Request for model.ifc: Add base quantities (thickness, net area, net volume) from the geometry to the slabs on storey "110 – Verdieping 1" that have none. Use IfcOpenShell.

First a look at what the model holds.

```python
import ifcopenshell
import ifcopenshell.util.element
import ifcopenshell.util.unit

model = ifcopenshell.open("model.ifc")
print(model.schema)
for unit_type in ("LENGTHUNIT", "AREAUNIT", "VOLUMEUNIT"):
    print(unit_type, ifcopenshell.util.unit.calculate_unit_scale(model, unit_type))
storey = next(s for s in model.by_type("IfcBuildingStorey") if s.Name == "110 – Verdieping 1")
slabs = [e for e in ifcopenshell.util.element.get_decomposition(storey) if e.is_a("IfcSlab")]
for e in sorted(slabs, key=lambda e: e.id()):
    print(e.id(), e.is_a(), e.Name, list(ifcopenshell.util.element.get_psets(e, qtos_only=True)), sep=" | ")
```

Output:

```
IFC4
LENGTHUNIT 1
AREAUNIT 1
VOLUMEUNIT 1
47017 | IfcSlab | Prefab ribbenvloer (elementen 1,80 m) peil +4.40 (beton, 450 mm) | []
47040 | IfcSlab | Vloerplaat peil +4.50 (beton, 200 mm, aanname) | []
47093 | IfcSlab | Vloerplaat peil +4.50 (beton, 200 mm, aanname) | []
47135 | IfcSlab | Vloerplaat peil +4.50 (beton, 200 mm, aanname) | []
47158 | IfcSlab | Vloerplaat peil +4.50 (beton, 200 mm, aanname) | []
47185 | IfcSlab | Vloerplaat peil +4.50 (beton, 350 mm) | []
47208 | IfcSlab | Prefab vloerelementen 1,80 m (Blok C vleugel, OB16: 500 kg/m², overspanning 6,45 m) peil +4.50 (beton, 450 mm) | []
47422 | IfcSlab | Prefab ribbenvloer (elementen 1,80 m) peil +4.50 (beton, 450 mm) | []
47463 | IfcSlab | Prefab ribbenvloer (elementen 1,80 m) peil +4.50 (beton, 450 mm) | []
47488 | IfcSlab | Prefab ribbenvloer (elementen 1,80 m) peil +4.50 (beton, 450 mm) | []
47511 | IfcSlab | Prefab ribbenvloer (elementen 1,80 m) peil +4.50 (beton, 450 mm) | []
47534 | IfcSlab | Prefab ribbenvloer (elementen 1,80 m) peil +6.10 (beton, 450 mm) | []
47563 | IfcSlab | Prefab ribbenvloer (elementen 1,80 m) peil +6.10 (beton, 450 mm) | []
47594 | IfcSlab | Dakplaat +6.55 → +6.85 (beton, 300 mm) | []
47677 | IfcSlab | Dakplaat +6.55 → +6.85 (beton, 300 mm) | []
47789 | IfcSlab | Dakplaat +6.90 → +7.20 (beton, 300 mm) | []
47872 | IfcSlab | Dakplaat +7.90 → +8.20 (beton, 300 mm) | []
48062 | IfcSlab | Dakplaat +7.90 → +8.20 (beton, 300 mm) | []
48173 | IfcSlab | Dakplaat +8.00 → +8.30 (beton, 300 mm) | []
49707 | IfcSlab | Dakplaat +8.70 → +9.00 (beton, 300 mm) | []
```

```python
import ifcopenshell
import ifcopenshell.api.pset
import ifcopenshell.geom
import ifcopenshell.util.element
import ifcopenshell.util.shape
import ifcopenshell.util.unit

model = ifcopenshell.open("model.ifc")
unit_scale = ifcopenshell.util.unit.calculate_unit_scale(model)
area_scale = ifcopenshell.util.unit.calculate_unit_scale(model, "AREAUNIT")
volume_scale = ifcopenshell.util.unit.calculate_unit_scale(model, "VOLUMEUNIT")
settings = ifcopenshell.geom.settings()

storey = next(s for s in model.by_type("IfcBuildingStorey") if s.Name == "110 – Verdieping 1")
slabs = [e for e in ifcopenshell.util.element.get_decomposition(storey) if e.is_a("IfcSlab")]

for e in sorted(slabs, key=lambda e: e.id()):
    if ifcopenshell.util.element.get_psets(e, qtos_only=True, should_inherit=False):
        continue
    # Geometry comes back in metres, in the element's own axes.
    shape = ifcopenshell.geom.create_shape(settings, e)
    values = {
        "Width": ifcopenshell.util.shape.get_z(shape.geometry) / unit_scale,
        "NetArea": ifcopenshell.util.shape.get_footprint_area(shape.geometry) / area_scale,
        "NetVolume": ifcopenshell.util.shape.get_volume(shape.geometry) / volume_scale,
    }
    qto = ifcopenshell.api.pset.add_qto(model, product=e, name="Qto_SlabBaseQuantities")
    ifcopenshell.api.pset.edit_qto(model, qto=qto, properties=values)
    print(e.id(), {k: round(v, 3) for k, v in values.items()})

model.write("model_updated.ifc")
```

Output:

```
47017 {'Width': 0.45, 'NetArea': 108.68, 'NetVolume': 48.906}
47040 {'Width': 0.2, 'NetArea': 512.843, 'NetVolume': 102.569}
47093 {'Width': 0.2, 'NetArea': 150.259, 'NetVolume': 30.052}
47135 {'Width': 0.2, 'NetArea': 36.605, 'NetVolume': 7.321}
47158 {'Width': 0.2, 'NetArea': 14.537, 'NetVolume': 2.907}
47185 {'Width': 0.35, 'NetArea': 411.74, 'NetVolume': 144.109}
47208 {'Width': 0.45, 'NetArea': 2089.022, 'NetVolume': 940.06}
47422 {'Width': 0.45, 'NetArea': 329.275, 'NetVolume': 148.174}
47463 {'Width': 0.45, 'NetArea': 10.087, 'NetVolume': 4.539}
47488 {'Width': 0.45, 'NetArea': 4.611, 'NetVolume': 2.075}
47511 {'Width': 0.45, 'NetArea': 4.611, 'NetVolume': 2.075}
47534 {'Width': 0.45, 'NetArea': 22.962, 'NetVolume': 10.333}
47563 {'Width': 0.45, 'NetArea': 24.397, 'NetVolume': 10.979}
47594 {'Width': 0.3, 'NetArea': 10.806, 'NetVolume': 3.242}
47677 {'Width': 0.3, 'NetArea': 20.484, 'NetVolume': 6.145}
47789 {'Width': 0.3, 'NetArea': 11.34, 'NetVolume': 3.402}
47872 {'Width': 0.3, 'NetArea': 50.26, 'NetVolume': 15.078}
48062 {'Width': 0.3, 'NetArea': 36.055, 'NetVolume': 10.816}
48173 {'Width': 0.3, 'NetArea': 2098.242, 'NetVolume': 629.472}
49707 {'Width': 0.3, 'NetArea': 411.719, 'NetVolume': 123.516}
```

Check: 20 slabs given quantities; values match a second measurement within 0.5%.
